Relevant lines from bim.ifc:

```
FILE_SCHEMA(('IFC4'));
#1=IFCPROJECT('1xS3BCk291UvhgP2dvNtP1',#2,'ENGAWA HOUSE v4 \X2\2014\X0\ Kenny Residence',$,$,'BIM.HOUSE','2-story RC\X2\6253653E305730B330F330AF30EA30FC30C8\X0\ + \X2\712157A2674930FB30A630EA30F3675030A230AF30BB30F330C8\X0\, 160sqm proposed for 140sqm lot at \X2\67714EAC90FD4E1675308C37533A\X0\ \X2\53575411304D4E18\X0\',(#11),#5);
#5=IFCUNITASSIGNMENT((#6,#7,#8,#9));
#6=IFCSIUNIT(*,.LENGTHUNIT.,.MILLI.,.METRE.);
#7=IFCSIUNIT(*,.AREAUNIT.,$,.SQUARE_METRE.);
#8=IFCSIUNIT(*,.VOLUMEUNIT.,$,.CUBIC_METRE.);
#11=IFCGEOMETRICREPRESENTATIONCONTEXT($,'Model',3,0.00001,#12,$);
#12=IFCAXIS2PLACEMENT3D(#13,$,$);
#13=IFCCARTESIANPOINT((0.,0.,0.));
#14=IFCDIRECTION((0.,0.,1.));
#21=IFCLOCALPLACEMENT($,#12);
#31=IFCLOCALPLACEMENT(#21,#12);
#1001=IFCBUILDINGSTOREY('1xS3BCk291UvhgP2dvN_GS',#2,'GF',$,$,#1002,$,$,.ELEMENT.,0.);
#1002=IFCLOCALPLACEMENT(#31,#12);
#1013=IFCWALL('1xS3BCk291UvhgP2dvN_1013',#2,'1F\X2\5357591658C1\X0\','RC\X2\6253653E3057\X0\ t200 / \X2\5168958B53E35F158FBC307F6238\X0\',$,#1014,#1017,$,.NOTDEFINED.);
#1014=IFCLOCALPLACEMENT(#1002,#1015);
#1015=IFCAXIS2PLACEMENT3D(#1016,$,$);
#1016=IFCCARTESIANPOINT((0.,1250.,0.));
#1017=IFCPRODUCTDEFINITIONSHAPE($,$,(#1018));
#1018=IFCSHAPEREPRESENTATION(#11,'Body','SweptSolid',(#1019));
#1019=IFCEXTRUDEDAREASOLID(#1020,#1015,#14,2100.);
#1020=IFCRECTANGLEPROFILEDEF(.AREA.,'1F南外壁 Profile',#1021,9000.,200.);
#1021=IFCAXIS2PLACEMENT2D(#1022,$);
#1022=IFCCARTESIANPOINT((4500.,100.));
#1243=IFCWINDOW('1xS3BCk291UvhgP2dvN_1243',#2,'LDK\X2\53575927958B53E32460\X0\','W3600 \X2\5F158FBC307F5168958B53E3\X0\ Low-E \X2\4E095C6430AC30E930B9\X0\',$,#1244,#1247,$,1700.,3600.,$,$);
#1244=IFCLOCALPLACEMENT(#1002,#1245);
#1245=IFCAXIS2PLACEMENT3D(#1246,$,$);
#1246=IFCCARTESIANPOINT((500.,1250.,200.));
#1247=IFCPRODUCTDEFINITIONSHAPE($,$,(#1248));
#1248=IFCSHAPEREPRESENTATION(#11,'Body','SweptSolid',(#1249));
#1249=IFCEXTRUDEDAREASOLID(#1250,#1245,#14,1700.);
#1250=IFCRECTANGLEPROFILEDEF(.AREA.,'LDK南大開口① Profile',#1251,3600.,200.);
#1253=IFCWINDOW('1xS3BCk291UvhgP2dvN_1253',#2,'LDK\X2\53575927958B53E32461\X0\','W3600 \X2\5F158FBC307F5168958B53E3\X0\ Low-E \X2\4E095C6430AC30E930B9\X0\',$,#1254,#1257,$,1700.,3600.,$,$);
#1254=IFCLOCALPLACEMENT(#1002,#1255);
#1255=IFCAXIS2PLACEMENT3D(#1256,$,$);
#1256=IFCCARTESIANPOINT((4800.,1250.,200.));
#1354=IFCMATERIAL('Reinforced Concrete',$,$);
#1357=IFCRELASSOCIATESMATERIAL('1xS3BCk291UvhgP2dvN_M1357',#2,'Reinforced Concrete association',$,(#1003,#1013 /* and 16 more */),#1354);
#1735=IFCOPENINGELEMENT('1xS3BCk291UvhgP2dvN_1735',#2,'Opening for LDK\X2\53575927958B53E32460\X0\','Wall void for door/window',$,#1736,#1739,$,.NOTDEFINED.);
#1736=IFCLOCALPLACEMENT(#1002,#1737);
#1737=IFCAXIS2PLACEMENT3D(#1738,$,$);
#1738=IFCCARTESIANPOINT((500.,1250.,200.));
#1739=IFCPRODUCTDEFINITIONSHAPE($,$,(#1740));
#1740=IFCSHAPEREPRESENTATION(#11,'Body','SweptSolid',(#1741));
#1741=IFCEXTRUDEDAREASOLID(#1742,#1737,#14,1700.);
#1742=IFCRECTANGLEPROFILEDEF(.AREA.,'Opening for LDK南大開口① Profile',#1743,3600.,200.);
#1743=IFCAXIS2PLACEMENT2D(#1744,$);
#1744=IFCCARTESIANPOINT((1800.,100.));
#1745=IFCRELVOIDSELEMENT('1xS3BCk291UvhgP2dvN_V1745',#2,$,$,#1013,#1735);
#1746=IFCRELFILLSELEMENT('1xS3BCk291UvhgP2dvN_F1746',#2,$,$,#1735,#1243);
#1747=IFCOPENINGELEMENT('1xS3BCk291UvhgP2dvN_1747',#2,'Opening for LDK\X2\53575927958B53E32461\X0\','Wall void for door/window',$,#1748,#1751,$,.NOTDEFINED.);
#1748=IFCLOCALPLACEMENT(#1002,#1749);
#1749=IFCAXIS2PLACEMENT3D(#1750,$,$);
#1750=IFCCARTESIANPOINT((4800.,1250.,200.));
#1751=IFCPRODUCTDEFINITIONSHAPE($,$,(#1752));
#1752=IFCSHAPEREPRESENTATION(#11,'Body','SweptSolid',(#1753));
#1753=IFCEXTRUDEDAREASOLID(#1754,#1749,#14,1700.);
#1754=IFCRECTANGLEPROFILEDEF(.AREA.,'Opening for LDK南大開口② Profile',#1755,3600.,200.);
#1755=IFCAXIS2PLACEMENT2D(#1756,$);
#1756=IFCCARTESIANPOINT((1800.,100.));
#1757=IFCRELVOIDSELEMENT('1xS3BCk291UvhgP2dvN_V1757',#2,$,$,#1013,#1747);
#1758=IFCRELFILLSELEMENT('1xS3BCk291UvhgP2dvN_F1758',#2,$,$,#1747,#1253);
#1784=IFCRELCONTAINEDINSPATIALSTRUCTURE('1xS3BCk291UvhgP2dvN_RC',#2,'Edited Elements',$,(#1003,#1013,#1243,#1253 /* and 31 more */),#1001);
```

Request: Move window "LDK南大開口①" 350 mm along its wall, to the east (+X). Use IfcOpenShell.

```python
import ifcopenshell
import ifcopenshell.api.geometry
import ifcopenshell.util.placement

model = ifcopenshell.open("bim.ifc")

window = model.by_guid("1xS3BCk291UvhgP2dvN_1243")
opening = window.FillsVoids[0].RelatingOpeningElement
wall = opening.VoidsElements[0].RelatingBuildingElement

wall_matrix = ifcopenshell.util.placement.get_local_placement(wall.ObjectPlacement)
shift = wall_matrix[:3, 0] * 350.0
before = ifcopenshell.util.placement.get_local_placement(window.ObjectPlacement)[:3, 3].copy()

# The window is not placed relative to its opening, so move both.
for product in (opening, window):
    matrix = ifcopenshell.util.placement.get_local_placement(product.ObjectPlacement)
    matrix[:3, 3] += shift
    ifcopenshell.api.geometry.edit_object_placement(model, product=product, matrix=matrix, is_si=False)

after = ifcopenshell.util.placement.get_local_placement(window.ObjectPlacement)[:3, 3]
print("window moved by", (after - before).round(3) + 0.0)

model.write("bim_v2.ifc")
```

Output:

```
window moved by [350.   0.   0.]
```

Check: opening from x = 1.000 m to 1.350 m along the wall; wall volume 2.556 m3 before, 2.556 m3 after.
